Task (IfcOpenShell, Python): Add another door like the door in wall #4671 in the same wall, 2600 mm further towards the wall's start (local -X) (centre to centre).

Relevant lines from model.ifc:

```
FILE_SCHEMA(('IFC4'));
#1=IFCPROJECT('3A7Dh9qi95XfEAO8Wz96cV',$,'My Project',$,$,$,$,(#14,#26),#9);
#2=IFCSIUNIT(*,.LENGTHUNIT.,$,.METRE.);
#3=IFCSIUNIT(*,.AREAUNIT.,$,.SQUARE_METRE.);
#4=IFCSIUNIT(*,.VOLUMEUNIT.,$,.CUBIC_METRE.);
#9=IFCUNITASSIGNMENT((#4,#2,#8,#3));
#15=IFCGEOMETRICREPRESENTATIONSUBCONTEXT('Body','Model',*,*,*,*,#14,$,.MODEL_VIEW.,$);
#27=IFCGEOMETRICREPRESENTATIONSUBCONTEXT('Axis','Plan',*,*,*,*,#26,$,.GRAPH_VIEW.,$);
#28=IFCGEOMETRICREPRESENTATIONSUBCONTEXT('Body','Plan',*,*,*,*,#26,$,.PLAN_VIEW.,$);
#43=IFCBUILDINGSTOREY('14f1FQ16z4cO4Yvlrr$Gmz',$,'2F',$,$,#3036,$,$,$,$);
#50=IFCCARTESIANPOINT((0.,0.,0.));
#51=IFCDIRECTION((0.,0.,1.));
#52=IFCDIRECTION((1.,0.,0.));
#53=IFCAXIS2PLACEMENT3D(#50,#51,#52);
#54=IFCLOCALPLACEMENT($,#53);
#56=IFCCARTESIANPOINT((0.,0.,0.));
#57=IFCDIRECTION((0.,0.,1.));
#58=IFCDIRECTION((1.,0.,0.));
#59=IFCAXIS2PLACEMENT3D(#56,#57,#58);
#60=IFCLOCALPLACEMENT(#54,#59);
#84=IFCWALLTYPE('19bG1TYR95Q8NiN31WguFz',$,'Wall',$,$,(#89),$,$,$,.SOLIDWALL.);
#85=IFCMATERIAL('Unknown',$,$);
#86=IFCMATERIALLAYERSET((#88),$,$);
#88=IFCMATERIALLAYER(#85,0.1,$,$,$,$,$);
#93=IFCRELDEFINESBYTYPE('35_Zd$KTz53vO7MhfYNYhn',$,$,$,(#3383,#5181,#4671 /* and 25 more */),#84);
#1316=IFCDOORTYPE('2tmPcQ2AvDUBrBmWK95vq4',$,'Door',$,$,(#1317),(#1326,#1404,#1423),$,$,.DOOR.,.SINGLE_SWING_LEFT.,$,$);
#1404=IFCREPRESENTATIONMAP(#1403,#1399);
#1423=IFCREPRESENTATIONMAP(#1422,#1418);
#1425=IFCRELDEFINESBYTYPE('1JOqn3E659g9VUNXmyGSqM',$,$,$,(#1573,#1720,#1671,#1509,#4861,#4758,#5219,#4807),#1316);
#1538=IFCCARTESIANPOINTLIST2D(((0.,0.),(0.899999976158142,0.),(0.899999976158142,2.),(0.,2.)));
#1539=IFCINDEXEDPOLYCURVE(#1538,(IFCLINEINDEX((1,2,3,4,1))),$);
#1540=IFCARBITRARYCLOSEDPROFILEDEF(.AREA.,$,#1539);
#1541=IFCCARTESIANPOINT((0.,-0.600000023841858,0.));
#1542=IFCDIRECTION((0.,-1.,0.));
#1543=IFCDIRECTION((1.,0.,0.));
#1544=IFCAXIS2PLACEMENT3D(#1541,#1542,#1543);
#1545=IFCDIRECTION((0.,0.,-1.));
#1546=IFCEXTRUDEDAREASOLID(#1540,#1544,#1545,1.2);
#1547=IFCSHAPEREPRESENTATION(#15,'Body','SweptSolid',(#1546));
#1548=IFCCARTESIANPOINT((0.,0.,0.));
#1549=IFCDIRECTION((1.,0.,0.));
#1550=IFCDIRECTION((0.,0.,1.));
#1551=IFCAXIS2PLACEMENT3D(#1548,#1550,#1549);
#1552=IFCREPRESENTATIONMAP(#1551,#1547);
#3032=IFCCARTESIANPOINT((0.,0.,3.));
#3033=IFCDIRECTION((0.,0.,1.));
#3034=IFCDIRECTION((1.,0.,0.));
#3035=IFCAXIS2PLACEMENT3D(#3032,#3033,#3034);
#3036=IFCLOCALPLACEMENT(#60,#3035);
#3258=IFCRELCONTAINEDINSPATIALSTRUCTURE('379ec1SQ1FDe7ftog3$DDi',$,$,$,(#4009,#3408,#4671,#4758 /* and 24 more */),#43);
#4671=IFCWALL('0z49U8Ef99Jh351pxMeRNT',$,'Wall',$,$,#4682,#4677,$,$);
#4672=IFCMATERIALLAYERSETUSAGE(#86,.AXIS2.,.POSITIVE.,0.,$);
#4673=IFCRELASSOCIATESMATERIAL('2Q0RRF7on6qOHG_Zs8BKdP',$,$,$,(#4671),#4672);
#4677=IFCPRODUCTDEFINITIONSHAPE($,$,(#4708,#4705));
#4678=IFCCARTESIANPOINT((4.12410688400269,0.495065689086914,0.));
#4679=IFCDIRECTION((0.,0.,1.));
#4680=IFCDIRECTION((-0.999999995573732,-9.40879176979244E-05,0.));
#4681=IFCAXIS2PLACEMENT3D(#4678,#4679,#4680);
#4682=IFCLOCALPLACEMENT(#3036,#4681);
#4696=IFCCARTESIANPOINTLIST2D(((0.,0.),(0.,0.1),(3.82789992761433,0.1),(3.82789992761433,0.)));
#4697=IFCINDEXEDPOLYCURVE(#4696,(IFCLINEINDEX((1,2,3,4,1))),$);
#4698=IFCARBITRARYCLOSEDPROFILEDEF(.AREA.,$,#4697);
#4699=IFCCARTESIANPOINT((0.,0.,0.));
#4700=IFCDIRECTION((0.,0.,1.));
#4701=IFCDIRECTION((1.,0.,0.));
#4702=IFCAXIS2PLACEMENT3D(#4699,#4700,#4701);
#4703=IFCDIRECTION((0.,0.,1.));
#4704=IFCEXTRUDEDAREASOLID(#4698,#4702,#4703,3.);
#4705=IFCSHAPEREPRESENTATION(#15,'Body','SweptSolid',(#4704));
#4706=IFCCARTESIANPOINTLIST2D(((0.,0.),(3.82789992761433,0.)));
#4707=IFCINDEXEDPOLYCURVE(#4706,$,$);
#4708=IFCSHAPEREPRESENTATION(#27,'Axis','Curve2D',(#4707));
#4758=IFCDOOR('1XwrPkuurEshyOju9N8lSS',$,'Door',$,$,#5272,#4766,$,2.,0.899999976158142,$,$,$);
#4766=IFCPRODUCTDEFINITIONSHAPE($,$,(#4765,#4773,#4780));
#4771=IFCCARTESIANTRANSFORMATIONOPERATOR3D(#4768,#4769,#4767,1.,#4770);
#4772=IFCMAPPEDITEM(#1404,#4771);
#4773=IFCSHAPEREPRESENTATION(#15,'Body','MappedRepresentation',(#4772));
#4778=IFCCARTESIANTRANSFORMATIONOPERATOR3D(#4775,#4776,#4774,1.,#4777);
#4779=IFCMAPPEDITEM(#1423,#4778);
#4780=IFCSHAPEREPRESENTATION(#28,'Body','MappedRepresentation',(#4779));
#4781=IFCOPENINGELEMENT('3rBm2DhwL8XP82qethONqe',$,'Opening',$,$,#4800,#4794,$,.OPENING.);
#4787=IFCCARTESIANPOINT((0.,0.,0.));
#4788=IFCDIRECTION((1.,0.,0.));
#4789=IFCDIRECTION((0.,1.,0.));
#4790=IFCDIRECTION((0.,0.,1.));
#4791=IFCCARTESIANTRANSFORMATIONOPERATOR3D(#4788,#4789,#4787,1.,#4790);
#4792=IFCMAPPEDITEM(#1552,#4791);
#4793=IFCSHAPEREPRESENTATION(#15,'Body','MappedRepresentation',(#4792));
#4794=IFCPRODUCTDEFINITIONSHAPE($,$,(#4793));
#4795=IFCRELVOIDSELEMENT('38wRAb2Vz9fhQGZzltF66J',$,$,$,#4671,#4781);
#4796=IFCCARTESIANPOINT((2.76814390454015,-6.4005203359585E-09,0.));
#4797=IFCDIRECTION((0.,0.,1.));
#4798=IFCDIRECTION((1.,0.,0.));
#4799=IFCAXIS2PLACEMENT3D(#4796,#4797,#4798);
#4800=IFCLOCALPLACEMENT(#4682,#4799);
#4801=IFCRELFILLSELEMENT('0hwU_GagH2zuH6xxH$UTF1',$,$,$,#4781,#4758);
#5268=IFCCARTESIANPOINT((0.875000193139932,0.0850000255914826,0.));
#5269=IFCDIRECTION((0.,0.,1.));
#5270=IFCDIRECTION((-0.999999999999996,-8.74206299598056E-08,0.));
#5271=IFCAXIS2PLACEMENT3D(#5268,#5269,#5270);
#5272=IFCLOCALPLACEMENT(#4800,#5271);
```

```python
import ifcopenshell
import ifcopenshell.api.feature
import ifcopenshell.api.geometry
import ifcopenshell.api.root
import ifcopenshell.geom
import ifcopenshell.util.element
import ifcopenshell.util.placement
import ifcopenshell.util.shape
import ifcopenshell.util.unit

model = ifcopenshell.open("model.ifc")
unit_scale = ifcopenshell.util.unit.calculate_unit_scale(model)
settings = ifcopenshell.geom.settings()


def volume(element):
    """Net volume in cubic metres, openings subtracted."""
    shape = ifcopenshell.geom.create_shape(settings, element)
    return ifcopenshell.util.shape.get_volume(shape.geometry)


door = model.by_id(4758)
opening = door.FillsVoids[0].RelatingOpeningElement
wall = opening.VoidsElements[0].RelatingBuildingElement
before = volume(wall)
shift = ifcopenshell.util.placement.get_local_placement(wall.ObjectPlacement)[:3, 0] * -2.6 / unit_scale

# copy_class copies the void relationship, type, container and properties, but no geometry.
new_opening = ifcopenshell.api.root.copy_class(model, product=opening)
new_opening.Representation = ifcopenshell.util.element.copy_deep(
    model, opening.Representation, exclude=["IfcGeometricRepresentationContext", "IfcRepresentationMap"]
)
new_door = ifcopenshell.api.root.copy_class(model, product=door)
new_door.Representation = ifcopenshell.util.element.copy_deep(
    model, door.Representation, exclude=["IfcGeometricRepresentationContext", "IfcRepresentationMap"]
)
ifcopenshell.api.feature.add_filling(model, opening=new_opening, element=new_door)

for old, new in ((opening, new_opening), (door, new_door)):
    matrix = ifcopenshell.util.placement.get_local_placement(old.ObjectPlacement)
    matrix[:3, 3] += shift
    ifcopenshell.api.geometry.edit_object_placement(model, product=new, matrix=matrix, is_si=False)

after = volume(wall)

print(f"wall volume {before:.3f} -> {after:.3f} m3")

model.write("model_v2.ifc")
```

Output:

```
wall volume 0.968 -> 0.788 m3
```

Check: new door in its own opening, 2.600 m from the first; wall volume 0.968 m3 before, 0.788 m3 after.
